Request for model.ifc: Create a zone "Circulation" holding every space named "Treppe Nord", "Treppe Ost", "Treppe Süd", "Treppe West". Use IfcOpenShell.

First a look at what the model holds.

```python
import ifcopenshell

model = ifcopenshell.open("model.ifc")
print(model.schema)
seen = {}
for space in model.by_type("IfcSpace"):
    seen[space.LongName] = seen.get(space.LongName, 0) + 1
for name, count in sorted(seen.items(), key=str):
    print(count, "x", name)
print("zones:", [z.Name for z in model.by_type("IfcZone")][:20])
```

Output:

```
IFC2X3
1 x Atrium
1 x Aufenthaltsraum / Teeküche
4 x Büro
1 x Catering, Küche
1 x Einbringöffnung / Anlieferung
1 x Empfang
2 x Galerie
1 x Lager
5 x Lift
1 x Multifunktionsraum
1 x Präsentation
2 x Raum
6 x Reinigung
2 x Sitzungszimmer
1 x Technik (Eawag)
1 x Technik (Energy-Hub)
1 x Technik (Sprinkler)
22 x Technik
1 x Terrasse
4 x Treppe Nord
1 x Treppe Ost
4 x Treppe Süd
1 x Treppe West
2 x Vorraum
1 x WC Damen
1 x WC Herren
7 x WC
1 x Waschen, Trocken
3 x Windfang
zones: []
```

```python
import ifcopenshell
import ifcopenshell.api.group
import ifcopenshell.api.root

model = ifcopenshell.open("model.ifc")

names = {"Treppe Nord", "Treppe Ost", "Treppe Süd", "Treppe West"}
spaces = [s for s in model.by_type("IfcSpace") if s.LongName in names]

zone = ifcopenshell.api.root.create_entity(model, ifc_class="IfcZone", name="Circulation")
ifcopenshell.api.group.assign_group(model, products=spaces, group=zone)
print(len(spaces), "spaces in", zone.Name)

model.write("model_updated.ifc")
```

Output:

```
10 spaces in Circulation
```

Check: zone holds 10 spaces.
